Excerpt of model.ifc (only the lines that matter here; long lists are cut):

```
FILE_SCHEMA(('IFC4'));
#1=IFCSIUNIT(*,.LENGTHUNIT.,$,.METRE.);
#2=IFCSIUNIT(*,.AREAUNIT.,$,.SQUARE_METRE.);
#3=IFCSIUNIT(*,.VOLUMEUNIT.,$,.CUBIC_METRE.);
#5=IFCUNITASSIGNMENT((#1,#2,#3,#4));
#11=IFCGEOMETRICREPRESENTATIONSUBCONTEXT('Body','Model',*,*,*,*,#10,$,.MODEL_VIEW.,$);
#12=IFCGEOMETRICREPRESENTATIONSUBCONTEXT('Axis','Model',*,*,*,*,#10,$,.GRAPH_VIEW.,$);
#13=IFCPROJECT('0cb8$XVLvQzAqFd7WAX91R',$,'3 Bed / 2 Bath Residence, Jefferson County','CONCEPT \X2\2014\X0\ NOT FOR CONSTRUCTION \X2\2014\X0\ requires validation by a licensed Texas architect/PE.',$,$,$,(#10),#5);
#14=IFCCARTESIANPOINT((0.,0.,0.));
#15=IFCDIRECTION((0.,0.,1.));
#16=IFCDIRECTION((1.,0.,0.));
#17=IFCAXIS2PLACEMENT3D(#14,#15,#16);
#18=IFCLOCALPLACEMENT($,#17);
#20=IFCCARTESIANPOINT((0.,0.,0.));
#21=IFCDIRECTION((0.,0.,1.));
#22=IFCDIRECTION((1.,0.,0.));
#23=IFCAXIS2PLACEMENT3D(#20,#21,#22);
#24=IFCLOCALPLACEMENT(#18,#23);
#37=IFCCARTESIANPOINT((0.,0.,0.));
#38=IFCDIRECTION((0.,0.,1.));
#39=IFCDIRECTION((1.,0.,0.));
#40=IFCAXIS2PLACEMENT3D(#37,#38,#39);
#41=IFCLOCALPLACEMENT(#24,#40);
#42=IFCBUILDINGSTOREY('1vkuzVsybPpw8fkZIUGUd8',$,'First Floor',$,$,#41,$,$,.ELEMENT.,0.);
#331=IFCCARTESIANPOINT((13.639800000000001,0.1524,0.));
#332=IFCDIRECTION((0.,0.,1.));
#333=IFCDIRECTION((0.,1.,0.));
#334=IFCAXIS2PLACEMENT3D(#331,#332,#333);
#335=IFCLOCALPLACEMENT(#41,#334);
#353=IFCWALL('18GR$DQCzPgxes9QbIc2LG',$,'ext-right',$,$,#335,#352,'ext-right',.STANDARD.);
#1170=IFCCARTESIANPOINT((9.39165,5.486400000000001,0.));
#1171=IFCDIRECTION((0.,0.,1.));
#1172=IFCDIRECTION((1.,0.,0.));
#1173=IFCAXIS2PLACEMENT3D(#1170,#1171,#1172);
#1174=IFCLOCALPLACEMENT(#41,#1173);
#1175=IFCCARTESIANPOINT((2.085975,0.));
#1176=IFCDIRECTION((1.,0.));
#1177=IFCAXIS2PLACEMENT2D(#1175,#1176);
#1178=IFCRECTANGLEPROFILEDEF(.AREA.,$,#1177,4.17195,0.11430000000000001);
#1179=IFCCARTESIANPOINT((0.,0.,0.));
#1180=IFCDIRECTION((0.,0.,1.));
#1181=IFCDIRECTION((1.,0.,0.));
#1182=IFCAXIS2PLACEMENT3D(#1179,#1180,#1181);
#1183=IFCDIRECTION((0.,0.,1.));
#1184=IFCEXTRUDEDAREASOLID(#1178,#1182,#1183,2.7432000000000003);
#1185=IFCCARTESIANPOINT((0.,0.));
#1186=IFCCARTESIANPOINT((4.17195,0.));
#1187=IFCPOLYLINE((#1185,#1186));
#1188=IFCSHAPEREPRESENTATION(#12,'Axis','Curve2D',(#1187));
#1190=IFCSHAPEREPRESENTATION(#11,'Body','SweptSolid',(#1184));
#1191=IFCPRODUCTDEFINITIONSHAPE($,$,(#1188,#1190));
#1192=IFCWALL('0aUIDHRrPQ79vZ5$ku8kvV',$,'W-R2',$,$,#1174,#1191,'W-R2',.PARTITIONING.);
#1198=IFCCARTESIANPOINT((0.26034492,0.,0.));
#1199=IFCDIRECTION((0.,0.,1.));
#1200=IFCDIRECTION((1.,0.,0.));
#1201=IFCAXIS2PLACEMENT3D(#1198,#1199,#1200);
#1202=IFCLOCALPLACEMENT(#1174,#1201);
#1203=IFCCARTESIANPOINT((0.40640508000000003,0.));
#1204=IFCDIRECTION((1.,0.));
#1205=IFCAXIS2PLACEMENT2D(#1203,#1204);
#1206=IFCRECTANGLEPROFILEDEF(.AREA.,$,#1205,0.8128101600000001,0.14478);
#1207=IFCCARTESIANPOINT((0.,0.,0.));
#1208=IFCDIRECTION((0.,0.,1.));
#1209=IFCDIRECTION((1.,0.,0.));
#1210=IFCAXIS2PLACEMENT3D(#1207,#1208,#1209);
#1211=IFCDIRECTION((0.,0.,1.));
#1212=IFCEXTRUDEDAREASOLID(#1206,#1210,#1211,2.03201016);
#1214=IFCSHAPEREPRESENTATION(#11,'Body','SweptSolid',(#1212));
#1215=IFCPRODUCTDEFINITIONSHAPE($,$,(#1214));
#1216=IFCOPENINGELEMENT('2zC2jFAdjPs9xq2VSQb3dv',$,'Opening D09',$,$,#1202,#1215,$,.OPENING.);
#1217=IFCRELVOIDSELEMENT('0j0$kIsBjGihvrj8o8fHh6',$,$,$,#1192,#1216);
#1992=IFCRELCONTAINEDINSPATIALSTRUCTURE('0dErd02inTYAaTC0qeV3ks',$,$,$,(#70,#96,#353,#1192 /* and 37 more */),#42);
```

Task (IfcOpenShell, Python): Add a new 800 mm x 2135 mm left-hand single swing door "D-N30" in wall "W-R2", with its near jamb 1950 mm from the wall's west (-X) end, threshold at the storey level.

```python
import numpy as np
import ifcopenshell
import ifcopenshell.api.feature
import ifcopenshell.api.geometry
import ifcopenshell.api.root
import ifcopenshell.api.spatial
import ifcopenshell.geom
import ifcopenshell.util.element
import ifcopenshell.util.placement
import ifcopenshell.util.representation
import ifcopenshell.util.shape
import ifcopenshell.util.unit

model = ifcopenshell.open("model.ifc")
unit_scale = ifcopenshell.util.unit.calculate_unit_scale(model)
settings = ifcopenshell.geom.settings()


def volume(element):
    """Net volume in cubic metres, openings subtracted."""
    shape = ifcopenshell.geom.create_shape(settings, element)
    return ifcopenshell.util.shape.get_volume(shape.geometry)


wall = model.by_id(1192)
storey = ifcopenshell.util.element.get_container(wall, ifc_class="IfcBuildingStorey")
context = ifcopenshell.util.representation.get_context(model, "Model", "Body", "MODEL_VIEW")
before = volume(wall)

width, height, from_end, sill = 0.8, 2.135, 1.95, 0.0  # metres

# The wall runs along its own X axis, and the end named is its -X end.
wall_shape = ifcopenshell.geom.create_shape(settings, wall)
x, y, z = ifcopenshell.util.shape.get_vertices(wall_shape.geometry).T
start = x.min() + from_end
face, thickness = float(y.min()), float(y.max() - y.min())
wall_matrix = ifcopenshell.util.placement.get_local_placement(wall.ObjectPlacement)
level = ifcopenshell.util.placement.get_local_placement(storey.ObjectPlacement)[2, 3]


def in_wall(x, y):
    """Placement at x, y metres in the wall's axes, at sill height."""
    matrix = wall_matrix.copy()
    matrix[:, 3] = wall_matrix @ np.array([x / unit_scale, y / unit_scale, 0.0, 1.0])
    matrix[2, 3] = level + sill / unit_scale
    return matrix


# Opening: a box that overshoots both wall faces by 50 mm.
opening = ifcopenshell.api.root.create_entity(model, ifc_class="IfcOpeningElement", predefined_type="OPENING")
box = ifcopenshell.api.geometry.add_wall_representation(
    model, context=context, length=width, height=height, thickness=thickness + 0.1
)
ifcopenshell.api.geometry.assign_representation(model, product=opening, representation=box)
ifcopenshell.api.geometry.edit_object_placement(model, product=opening, matrix=in_wall(start, face - 0.05), is_si=False)
ifcopenshell.api.feature.add_feature(model, feature=opening, element=wall)

door = ifcopenshell.api.root.create_entity(model, ifc_class="IfcDoor", name="D-N30", predefined_type="DOOR")
door.OverallWidth, door.OverallHeight = width / unit_scale, height / unit_scale
door.OperationType = "SINGLE_SWING_LEFT"
body = ifcopenshell.api.geometry.add_door_representation(
    model,
    context=context,
    overall_width=door.OverallWidth,
    overall_height=door.OverallHeight,
    operation_type="SINGLE_SWING_LEFT",
    lining_properties={"LiningDepth": thickness / unit_scale, "ThresholdDepth": thickness / unit_scale},
)
ifcopenshell.api.geometry.assign_representation(model, product=door, representation=body)
ifcopenshell.api.spatial.assign_container(model, products=[door], relating_structure=storey)
ifcopenshell.api.feature.add_filling(model, opening=opening, element=door)

# The lining spans the wall, so the door starts at the wall face.
ifcopenshell.api.geometry.edit_object_placement(model, product=door, matrix=in_wall(start, face), is_si=False)

after = volume(wall)

print(f"wall volume {before:.3f} -> {after:.3f} m3")

model.write("model_updated.ifc")
```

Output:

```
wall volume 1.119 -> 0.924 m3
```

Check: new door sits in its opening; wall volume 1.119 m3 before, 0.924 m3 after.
